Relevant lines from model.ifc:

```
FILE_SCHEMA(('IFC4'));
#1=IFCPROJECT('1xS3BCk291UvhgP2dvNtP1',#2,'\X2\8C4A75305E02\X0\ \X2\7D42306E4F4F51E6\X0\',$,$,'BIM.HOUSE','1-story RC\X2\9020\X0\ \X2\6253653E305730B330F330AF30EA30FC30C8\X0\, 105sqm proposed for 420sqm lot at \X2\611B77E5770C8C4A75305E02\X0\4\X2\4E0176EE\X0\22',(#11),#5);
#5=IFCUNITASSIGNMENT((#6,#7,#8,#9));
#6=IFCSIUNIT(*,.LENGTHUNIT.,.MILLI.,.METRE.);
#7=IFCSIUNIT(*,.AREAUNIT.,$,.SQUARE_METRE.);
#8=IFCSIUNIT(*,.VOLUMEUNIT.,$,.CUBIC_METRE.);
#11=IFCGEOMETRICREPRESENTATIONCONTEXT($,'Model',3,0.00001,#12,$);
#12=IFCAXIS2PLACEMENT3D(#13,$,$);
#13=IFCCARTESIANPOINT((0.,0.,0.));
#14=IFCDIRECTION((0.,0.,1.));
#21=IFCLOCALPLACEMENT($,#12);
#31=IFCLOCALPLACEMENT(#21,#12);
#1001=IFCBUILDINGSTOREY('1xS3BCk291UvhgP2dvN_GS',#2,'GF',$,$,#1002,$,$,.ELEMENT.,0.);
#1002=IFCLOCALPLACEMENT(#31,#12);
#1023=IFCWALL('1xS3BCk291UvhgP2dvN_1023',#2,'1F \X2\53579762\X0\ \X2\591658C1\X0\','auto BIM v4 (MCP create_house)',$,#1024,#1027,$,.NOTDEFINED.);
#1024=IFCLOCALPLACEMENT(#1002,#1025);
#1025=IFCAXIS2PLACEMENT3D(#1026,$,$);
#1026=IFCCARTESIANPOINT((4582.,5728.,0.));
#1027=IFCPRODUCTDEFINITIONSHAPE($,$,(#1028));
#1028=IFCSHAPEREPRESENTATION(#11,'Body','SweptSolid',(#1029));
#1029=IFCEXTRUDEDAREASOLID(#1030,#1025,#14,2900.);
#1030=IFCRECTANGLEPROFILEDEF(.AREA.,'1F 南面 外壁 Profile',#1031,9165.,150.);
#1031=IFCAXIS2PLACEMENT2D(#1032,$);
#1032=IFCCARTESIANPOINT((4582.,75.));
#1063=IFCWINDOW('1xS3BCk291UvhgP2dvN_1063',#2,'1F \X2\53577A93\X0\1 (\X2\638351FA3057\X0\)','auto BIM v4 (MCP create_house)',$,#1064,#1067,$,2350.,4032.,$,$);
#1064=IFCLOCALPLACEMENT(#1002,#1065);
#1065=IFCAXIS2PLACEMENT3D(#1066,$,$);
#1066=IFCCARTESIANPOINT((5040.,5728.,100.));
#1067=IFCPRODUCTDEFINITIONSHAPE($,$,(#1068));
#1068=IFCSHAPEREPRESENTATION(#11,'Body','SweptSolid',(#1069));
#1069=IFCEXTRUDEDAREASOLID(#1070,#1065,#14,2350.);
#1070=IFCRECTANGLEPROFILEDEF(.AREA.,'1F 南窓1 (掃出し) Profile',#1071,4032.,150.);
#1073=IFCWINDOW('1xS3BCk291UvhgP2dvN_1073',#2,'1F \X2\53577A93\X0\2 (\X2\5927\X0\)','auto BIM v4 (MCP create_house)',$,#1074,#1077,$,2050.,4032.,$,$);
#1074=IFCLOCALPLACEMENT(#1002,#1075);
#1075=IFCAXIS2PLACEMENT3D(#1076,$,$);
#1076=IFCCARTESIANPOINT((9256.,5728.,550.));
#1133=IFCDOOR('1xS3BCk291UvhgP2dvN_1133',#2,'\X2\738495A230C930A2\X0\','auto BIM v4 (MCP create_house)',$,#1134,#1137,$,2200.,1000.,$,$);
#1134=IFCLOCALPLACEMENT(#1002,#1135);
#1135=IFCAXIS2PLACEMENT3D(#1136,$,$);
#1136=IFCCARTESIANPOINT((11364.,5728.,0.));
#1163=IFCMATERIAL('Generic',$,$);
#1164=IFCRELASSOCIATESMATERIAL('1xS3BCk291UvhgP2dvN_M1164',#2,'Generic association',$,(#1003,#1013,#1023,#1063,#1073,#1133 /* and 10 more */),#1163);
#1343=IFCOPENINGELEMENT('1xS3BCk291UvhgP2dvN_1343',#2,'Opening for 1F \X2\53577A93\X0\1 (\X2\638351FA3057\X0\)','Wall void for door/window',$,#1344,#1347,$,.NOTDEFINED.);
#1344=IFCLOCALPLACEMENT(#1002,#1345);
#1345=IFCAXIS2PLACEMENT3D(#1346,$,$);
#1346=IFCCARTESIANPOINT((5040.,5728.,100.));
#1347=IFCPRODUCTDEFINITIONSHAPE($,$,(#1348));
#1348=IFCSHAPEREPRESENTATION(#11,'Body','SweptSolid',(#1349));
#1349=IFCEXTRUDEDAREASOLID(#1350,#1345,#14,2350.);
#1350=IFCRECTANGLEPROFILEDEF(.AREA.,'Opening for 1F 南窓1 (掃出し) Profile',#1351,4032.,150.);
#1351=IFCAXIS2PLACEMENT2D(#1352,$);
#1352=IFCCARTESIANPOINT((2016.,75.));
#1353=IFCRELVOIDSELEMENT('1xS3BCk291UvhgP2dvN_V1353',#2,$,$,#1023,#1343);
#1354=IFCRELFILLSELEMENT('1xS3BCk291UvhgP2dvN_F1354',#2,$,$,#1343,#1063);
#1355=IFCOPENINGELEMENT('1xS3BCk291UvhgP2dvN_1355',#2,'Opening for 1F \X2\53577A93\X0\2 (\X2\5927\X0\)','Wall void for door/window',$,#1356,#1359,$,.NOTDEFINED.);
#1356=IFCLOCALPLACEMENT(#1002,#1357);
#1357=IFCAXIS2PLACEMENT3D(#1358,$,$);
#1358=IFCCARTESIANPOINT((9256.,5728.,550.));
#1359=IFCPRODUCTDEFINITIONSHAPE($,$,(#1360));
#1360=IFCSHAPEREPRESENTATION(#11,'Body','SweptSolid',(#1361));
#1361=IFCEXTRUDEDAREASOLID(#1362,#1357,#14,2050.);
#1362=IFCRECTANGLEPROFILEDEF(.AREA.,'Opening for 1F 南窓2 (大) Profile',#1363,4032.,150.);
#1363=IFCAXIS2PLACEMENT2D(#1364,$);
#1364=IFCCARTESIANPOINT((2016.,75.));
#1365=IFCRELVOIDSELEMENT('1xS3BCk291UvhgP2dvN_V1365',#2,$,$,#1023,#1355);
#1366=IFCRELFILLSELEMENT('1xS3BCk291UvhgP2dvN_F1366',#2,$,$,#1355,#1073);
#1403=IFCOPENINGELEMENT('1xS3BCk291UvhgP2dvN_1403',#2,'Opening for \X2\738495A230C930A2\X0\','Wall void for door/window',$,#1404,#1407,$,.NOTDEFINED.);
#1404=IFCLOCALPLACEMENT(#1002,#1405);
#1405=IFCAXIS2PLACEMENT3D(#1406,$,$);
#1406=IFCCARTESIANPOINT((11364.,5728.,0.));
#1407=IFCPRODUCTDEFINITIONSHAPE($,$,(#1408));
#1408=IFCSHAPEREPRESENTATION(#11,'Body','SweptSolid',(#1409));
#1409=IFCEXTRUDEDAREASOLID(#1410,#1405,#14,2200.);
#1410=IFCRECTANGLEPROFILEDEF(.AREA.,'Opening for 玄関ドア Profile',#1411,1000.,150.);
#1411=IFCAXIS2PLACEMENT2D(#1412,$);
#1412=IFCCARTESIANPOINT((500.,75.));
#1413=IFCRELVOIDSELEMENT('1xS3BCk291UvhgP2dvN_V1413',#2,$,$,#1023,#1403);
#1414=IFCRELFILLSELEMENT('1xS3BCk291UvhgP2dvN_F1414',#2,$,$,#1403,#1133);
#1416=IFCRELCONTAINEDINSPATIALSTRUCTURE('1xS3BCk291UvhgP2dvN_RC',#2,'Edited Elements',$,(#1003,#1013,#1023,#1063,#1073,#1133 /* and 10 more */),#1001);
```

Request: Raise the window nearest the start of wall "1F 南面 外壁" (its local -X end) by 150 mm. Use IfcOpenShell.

```python
import numpy as np
import ifcopenshell
import ifcopenshell.api.geometry
import ifcopenshell.util.placement
import ifcopenshell.util.unit

model = ifcopenshell.open("model.ifc")
unit_scale = ifcopenshell.util.unit.calculate_unit_scale(model)

window = model.by_guid("1xS3BCk291UvhgP2dvN_1063")
opening = window.FillsVoids[0].RelatingOpeningElement
dz = 150.0

shift = np.array([0.0, 0.0, dz])
# The window is not placed relative to its opening, so move both.
for product in (opening, window):
    matrix = ifcopenshell.util.placement.get_local_placement(product.ObjectPlacement)
    matrix[:3, 3] += shift
    ifcopenshell.api.geometry.edit_object_placement(model, product=product, matrix=matrix, is_si=False)

print(f"moved by {dz * unit_scale:+.3f} m")

model.write("model_updated.ifc")
```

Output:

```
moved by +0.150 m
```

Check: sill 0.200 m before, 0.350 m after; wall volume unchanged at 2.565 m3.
